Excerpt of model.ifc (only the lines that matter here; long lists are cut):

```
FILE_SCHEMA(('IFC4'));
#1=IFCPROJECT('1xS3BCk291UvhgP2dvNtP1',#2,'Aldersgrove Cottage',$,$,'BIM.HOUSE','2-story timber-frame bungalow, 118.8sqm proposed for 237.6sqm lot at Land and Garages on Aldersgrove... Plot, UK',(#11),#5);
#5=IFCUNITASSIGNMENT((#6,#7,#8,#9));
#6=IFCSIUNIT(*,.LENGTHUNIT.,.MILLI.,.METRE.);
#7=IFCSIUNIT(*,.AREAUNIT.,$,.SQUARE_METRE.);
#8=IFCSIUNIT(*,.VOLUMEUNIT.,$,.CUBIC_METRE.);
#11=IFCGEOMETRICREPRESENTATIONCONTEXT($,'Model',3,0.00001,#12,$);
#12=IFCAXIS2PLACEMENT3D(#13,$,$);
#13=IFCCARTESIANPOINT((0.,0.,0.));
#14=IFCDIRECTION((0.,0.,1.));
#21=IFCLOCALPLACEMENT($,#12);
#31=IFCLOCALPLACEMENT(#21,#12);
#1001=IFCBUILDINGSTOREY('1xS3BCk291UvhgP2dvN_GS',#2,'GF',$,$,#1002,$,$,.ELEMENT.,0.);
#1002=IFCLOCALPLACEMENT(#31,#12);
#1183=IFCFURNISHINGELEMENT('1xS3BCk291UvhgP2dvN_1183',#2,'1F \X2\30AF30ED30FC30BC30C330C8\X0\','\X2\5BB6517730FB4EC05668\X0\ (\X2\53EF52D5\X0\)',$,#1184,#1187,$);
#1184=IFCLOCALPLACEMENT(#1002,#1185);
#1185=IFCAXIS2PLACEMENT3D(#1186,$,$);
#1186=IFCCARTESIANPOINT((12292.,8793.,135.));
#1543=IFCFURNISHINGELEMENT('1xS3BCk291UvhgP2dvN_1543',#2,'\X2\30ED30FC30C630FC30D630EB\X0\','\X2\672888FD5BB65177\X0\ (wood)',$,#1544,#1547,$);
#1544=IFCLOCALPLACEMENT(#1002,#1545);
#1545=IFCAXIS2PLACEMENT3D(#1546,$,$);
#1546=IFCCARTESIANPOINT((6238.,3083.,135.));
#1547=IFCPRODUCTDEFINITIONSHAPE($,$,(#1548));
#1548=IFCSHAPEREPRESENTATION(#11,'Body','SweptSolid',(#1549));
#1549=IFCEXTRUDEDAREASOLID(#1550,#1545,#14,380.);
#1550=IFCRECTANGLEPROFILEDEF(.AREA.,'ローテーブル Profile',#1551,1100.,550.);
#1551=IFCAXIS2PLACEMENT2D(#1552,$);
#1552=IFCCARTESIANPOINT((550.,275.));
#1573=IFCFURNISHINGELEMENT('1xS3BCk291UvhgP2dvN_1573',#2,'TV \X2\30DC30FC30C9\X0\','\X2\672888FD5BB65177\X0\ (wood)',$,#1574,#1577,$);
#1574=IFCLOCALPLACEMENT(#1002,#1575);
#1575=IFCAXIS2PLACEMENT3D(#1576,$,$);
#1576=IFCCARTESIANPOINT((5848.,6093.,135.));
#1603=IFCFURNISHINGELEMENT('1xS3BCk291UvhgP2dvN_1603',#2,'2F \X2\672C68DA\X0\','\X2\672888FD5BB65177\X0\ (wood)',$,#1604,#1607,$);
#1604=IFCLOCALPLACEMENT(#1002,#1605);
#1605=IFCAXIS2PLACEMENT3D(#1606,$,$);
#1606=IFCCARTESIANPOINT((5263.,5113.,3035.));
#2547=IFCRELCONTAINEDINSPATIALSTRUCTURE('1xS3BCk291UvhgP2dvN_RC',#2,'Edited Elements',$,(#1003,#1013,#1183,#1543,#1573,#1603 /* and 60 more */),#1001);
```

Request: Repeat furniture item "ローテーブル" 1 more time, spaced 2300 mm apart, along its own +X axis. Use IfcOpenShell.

```python
import ifcopenshell
import ifcopenshell.api.geometry
import ifcopenshell.api.root
import ifcopenshell.util.element
import ifcopenshell.util.placement
import ifcopenshell.util.unit

model = ifcopenshell.open("model.ifc")
unit_scale = ifcopenshell.util.unit.calculate_unit_scale(model)


def reuse_history(source, copy):
    """copy_class also copies each property set's owner history, people and application; keep the originals."""
    for rel in copy.IsDefinedBy:
        if rel.is_a("IfcRelDefinesByProperties") and (history := rel.RelatingPropertyDefinition.OwnerHistory):
            rel.RelatingPropertyDefinition.OwnerHistory = source.OwnerHistory
            ifcopenshell.util.element.remove_deep2(model, history)


source = model.by_guid("1xS3BCk291UvhgP2dvN_1543")
base = ifcopenshell.util.placement.get_local_placement(source.ObjectPlacement)
step = base[:3, 0] * 2.3 / unit_scale

for i in range(1, 2):
    copy = ifcopenshell.api.root.copy_class(model, product=source)
    copy.Representation = ifcopenshell.util.element.copy_deep(
        model, source.Representation, exclude=["IfcGeometricRepresentationContext", "IfcRepresentationMap"]
    )
    reuse_history(source, copy)
    matrix = base.copy()
    matrix[:3, 3] += i * step
    print("added at", matrix[:3, 3].round(3) + 0.0)
    ifcopenshell.api.geometry.edit_object_placement(model, product=copy, matrix=matrix, is_si=False)

model.write("model_rev.ifc")
```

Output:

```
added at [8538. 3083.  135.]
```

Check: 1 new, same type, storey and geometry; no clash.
